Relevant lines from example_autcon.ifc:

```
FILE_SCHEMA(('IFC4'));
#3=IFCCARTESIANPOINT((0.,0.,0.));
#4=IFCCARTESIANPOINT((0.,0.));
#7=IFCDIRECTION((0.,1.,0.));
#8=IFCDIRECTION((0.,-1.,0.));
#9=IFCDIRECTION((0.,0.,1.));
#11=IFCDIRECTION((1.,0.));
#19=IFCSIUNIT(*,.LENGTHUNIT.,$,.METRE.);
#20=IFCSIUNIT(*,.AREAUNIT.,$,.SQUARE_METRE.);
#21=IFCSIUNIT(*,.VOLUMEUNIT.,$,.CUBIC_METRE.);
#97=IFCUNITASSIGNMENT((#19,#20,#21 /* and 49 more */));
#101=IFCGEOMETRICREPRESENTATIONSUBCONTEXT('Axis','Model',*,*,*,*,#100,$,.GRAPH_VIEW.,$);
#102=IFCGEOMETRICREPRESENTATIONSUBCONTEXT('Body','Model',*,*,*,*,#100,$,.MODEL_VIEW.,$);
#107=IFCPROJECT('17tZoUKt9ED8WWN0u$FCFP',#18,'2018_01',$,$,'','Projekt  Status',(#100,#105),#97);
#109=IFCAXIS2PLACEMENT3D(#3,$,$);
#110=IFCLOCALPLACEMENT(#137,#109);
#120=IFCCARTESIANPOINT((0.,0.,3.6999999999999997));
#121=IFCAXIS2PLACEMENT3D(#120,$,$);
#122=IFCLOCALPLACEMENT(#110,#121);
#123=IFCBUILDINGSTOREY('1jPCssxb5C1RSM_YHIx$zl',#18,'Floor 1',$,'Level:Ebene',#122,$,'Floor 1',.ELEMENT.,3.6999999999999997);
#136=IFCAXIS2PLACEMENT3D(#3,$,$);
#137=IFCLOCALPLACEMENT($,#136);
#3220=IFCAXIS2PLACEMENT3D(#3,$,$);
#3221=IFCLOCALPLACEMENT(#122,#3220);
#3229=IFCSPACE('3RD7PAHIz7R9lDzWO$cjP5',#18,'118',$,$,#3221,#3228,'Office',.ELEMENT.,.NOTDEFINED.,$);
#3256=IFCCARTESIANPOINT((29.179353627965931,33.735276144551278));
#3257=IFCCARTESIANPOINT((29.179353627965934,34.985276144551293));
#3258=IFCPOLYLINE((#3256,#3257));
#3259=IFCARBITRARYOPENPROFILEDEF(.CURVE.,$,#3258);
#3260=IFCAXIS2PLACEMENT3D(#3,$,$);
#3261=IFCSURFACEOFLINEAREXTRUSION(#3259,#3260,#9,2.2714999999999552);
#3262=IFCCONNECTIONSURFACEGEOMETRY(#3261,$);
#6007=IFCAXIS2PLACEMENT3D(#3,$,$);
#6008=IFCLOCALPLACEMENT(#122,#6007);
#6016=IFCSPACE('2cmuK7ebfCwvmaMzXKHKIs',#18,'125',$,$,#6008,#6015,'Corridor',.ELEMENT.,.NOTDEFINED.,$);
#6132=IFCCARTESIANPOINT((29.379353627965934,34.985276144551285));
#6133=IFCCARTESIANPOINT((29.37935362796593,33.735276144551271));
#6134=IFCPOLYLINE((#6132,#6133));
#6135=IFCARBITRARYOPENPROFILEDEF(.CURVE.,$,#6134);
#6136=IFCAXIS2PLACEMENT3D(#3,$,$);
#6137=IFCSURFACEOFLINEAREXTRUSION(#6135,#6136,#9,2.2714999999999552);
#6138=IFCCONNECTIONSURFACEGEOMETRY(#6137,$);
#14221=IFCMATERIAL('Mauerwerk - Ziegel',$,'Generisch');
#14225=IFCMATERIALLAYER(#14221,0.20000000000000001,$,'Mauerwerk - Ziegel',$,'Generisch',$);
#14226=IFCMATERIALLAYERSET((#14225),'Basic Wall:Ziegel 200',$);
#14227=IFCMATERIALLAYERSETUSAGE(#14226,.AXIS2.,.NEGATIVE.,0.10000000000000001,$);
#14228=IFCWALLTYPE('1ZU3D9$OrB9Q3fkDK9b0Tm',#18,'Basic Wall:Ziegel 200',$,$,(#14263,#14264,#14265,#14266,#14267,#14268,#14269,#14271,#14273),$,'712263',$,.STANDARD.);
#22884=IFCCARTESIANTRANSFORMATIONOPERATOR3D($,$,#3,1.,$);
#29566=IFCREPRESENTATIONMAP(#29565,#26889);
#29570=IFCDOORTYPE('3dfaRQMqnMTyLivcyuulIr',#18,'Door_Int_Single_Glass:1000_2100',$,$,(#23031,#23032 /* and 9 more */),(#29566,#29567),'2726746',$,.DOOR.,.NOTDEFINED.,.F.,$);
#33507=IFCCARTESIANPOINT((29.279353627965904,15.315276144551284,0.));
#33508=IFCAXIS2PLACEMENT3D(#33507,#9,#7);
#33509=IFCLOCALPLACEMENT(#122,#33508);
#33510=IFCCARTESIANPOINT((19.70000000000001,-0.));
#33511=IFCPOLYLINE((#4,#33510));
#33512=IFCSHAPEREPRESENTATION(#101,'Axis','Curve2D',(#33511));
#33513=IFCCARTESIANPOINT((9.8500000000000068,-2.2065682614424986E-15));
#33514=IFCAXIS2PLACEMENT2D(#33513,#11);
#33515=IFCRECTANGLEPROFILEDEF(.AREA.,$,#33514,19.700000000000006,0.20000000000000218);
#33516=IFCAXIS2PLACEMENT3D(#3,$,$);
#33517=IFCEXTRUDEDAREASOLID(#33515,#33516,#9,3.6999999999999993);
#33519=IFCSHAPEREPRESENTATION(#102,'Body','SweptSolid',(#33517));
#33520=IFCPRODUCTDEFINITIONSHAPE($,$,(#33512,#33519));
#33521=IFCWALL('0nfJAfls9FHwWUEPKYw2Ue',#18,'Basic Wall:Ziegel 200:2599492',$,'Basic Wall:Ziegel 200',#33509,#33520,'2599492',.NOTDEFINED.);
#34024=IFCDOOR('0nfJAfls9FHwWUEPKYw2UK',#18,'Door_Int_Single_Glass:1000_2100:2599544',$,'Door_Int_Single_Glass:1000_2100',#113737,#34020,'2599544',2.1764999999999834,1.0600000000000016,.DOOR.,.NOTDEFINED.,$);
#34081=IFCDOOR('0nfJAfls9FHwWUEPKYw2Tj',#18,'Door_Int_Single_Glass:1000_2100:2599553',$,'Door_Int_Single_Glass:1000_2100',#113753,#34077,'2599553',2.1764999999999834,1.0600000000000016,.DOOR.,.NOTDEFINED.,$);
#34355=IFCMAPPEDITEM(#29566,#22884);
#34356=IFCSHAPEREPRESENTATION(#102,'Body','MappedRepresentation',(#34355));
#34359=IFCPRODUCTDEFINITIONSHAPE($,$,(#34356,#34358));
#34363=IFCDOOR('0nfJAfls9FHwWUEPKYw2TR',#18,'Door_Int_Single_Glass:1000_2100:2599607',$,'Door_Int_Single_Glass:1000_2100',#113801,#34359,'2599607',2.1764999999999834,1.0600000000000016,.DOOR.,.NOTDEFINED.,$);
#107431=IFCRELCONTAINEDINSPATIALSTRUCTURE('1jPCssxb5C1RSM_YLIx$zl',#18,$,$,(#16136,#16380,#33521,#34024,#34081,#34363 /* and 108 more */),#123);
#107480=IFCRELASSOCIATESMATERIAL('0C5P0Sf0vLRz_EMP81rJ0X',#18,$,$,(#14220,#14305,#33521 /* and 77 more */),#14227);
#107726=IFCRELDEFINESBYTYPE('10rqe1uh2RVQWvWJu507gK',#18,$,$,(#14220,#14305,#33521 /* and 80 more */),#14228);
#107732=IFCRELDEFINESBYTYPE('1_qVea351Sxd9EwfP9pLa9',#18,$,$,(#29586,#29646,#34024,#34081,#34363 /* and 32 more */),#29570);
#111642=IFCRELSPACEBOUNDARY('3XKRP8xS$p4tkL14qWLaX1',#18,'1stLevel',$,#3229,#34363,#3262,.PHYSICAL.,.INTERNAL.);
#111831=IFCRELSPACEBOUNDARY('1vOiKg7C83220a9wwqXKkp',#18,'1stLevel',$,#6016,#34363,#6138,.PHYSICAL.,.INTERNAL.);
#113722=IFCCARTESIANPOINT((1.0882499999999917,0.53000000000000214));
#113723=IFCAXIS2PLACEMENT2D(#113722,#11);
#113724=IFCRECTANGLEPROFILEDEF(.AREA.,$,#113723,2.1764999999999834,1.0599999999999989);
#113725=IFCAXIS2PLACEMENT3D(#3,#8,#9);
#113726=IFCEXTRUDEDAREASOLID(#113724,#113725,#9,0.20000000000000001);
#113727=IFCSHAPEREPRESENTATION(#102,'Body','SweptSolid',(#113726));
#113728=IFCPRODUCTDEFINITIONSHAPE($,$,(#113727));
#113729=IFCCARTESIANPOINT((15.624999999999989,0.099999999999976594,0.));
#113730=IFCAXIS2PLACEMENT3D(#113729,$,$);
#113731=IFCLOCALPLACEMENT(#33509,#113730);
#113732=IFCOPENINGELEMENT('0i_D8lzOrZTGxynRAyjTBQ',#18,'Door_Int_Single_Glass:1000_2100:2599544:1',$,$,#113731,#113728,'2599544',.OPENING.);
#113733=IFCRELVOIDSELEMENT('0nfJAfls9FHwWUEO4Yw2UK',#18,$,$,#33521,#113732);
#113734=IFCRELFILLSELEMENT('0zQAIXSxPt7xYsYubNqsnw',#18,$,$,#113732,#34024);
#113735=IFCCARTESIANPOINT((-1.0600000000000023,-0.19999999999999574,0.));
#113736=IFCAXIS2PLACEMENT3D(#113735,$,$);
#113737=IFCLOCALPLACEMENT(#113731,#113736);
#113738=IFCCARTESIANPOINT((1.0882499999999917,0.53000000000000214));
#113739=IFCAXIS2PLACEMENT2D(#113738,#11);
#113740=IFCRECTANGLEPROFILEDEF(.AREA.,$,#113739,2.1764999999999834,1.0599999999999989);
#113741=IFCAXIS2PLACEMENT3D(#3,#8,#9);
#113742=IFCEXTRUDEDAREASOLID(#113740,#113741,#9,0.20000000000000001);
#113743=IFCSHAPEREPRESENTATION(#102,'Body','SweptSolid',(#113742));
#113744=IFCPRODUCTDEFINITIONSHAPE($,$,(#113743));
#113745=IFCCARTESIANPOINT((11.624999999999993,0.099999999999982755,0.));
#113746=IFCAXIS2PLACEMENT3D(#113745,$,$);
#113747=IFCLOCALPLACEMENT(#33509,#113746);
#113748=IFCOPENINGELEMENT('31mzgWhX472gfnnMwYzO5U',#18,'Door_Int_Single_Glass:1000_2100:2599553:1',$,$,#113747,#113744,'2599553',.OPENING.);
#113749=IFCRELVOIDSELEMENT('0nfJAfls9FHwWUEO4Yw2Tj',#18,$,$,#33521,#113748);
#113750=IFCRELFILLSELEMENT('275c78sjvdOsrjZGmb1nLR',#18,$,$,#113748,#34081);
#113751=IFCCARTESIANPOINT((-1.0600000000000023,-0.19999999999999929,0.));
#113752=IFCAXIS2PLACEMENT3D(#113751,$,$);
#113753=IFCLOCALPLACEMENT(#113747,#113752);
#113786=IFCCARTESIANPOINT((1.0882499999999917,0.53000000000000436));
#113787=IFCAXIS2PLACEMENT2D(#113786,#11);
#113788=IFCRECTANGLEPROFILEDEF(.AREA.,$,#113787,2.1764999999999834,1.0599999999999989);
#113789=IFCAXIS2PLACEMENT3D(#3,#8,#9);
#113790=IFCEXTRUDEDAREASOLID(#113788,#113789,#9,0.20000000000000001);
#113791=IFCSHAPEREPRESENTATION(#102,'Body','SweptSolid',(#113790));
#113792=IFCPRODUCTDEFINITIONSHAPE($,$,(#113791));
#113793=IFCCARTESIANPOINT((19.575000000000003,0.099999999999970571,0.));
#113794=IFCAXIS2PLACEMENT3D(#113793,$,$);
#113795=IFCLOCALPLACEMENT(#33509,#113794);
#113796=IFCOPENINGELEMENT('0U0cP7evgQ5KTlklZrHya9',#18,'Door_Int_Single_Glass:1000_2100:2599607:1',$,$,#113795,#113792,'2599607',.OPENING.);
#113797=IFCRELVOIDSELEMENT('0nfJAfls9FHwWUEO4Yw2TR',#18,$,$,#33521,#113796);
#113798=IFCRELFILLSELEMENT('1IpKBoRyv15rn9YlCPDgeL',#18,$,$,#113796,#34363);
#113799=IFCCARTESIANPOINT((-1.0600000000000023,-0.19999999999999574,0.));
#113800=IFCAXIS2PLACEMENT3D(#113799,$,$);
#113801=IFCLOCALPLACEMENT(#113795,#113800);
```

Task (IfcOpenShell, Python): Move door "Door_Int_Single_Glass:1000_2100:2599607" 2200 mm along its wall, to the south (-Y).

```python
import numpy as np
import ifcopenshell
import ifcopenshell.api.geometry
import ifcopenshell.util.placement
import ifcopenshell.util.unit

model = ifcopenshell.open("example_autcon.ifc")
unit_scale = ifcopenshell.util.unit.calculate_unit_scale(model)

door = model.by_id(34363)
opening = door.FillsVoids[0].RelatingOpeningElement
wall = opening.VoidsElements[0].RelatingBuildingElement

wall_matrix = ifcopenshell.util.placement.get_local_placement(wall.ObjectPlacement)
shift = wall_matrix[:3, 0] * -2.2 / unit_scale
before = ifcopenshell.util.placement.get_local_placement(door.ObjectPlacement)[:3, 3].copy()

# The door is placed relative to its opening, so it follows when the opening moves.
matrix = ifcopenshell.util.placement.get_local_placement(opening.ObjectPlacement)
matrix[:3, 3] += shift
ifcopenshell.api.geometry.edit_object_placement(
    model, product=opening, matrix=matrix, is_si=False, should_transform_children=True
)

# Space boundary surfaces are stored in each space's coordinates; move them too.
for rel in door.ProvidesBoundaries:
    if not rel.ConnectionGeometry:
        continue
    surface = rel.ConnectionGeometry.SurfaceOnRelatingElement
    space_matrix = ifcopenshell.util.placement.get_local_placement(rel.RelatingSpace.ObjectPlacement)
    point = np.array(surface.Position.Location.Coordinates) + space_matrix[:3, :3].T @ shift
    surface.Position = model.createIfcAxis2Placement3D(
        model.createIfcCartesianPoint(point.tolist()), surface.Position.Axis, surface.Position.RefDirection
    )

after = ifcopenshell.util.placement.get_local_placement(door.ObjectPlacement)[:3, 3]
print("door moved by", (after - before).round(3) + 0.0)

model.write("example_autcon_updated.ifc")
```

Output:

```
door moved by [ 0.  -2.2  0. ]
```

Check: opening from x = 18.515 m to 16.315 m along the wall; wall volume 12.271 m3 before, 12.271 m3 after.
